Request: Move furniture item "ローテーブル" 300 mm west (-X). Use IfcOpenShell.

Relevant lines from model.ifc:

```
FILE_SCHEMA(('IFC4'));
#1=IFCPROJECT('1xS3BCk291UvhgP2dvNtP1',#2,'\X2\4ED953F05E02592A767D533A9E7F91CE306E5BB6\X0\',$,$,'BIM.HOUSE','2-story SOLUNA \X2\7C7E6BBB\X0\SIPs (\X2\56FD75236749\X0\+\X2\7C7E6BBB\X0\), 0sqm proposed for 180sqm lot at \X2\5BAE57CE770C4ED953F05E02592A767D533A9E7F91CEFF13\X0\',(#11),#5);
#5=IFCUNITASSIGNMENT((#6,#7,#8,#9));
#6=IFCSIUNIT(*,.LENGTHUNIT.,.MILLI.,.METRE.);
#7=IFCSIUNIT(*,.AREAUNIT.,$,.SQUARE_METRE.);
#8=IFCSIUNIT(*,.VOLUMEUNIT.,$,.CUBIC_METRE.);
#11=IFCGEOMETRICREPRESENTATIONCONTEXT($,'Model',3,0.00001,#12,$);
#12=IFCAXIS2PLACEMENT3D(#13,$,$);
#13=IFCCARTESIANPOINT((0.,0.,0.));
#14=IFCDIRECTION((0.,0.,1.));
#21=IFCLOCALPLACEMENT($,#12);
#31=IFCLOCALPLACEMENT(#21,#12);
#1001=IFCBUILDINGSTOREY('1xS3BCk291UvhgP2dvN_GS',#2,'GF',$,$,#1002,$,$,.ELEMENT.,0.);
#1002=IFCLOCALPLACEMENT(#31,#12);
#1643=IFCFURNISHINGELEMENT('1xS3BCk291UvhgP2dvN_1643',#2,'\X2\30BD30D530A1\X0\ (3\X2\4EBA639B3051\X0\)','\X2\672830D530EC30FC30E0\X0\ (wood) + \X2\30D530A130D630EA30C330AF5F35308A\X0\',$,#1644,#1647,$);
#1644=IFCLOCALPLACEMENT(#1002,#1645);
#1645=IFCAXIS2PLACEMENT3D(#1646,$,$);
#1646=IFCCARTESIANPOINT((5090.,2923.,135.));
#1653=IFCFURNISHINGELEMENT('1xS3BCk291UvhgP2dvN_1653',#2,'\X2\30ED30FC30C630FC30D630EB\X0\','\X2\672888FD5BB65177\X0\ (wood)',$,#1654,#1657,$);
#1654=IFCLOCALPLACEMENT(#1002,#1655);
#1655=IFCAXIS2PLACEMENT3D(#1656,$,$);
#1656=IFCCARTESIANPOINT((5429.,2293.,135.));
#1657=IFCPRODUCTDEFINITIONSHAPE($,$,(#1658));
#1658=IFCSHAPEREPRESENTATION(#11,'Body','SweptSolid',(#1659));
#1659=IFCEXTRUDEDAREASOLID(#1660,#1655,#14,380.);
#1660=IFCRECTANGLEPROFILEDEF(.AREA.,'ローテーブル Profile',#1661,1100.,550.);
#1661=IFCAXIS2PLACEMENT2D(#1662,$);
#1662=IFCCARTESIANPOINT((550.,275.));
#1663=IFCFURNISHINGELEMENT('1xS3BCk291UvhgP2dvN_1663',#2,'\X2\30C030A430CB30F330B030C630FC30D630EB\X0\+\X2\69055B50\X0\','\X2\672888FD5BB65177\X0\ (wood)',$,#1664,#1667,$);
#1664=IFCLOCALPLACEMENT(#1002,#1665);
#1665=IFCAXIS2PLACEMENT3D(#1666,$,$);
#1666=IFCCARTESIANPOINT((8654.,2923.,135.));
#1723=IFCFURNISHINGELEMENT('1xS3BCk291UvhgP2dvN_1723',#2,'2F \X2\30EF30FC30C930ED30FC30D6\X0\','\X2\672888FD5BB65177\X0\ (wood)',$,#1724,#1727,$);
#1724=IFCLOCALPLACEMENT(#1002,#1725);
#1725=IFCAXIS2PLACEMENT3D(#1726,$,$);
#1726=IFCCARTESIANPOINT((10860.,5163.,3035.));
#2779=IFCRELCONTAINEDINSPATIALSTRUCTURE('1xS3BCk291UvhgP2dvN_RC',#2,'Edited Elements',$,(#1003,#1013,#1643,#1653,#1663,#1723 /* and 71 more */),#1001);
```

```python
import ifcopenshell
import ifcopenshell.api.geometry
import ifcopenshell.util.placement
import ifcopenshell.util.unit

model = ifcopenshell.open("model.ifc")
unit_scale = ifcopenshell.util.unit.calculate_unit_scale(model)

item = model.by_id(1653)
matrix = ifcopenshell.util.placement.get_local_placement(item.ObjectPlacement)
matrix[0, 3] -= 0.3 / unit_scale
ifcopenshell.api.geometry.edit_object_placement(model, product=item, matrix=matrix, is_si=False)

print(ifcopenshell.util.placement.get_local_placement(item.ObjectPlacement).round(3) + 0.0)

model.write("model_edited.ifc")
```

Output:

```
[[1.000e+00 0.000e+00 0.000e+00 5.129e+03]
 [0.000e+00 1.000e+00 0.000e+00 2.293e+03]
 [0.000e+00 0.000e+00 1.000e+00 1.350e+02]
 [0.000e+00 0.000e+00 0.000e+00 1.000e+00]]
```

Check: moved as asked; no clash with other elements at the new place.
